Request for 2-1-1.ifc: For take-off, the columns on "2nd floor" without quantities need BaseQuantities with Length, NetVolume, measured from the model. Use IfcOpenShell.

First a look at what the model holds.

```python
import ifcopenshell
import ifcopenshell.util.element
import ifcopenshell.util.unit

model = ifcopenshell.open("2-1-1.ifc")
print(model.schema)
for unit_type in ("LENGTHUNIT", "AREAUNIT", "VOLUMEUNIT"):
    print(unit_type, ifcopenshell.util.unit.calculate_unit_scale(model, unit_type))
storey = next(s for s in model.by_type("IfcBuildingStorey") if s.Name == "2nd floor")
columns = [e for e in ifcopenshell.util.element.get_decomposition(storey) if e.is_a("IfcColumn")]
for e in sorted(columns, key=lambda e: e.id()):
    print(e.id(), e.is_a(), e.Name, list(ifcopenshell.util.element.get_psets(e, qtos_only=True)), sep=" | ")
```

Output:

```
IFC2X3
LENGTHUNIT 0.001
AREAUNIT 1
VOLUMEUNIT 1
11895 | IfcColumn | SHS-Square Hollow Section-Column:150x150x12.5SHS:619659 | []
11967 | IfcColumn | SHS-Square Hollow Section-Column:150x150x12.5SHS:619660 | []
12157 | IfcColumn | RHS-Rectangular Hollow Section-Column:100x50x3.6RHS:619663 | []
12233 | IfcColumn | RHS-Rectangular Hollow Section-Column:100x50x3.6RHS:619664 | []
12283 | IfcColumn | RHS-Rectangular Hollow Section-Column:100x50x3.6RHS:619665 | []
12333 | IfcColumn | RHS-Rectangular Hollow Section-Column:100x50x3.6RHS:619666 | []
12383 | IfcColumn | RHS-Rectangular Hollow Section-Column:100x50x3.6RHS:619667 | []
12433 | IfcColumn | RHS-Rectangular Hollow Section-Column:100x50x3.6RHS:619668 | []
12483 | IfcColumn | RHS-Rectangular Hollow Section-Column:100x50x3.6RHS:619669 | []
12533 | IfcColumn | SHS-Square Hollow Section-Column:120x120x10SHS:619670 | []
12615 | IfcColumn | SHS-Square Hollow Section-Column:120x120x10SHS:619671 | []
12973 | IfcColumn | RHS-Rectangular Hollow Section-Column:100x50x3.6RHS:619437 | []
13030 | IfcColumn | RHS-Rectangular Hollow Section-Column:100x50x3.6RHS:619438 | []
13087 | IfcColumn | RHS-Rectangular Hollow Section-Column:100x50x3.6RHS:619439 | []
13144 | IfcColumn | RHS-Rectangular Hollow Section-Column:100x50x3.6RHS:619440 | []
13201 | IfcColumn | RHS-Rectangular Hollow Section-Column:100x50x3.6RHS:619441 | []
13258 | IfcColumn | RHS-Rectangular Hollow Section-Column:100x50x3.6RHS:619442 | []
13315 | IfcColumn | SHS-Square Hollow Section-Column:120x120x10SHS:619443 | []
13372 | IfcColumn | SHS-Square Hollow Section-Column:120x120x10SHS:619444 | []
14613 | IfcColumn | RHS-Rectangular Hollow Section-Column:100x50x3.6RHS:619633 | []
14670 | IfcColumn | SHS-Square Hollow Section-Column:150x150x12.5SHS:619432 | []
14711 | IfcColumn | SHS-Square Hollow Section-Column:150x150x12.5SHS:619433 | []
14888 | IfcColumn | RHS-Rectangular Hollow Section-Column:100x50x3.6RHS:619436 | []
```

```python
import ifcopenshell
import ifcopenshell.api.pset
import ifcopenshell.geom
import ifcopenshell.util.element
import ifcopenshell.util.shape
import ifcopenshell.util.unit

model = ifcopenshell.open("2-1-1.ifc")
unit_scale = ifcopenshell.util.unit.calculate_unit_scale(model)
volume_scale = ifcopenshell.util.unit.calculate_unit_scale(model, "VOLUMEUNIT")
settings = ifcopenshell.geom.settings()

storey = next(s for s in model.by_type("IfcBuildingStorey") if s.Name == "2nd floor")
columns = [e for e in ifcopenshell.util.element.get_decomposition(storey) if e.is_a("IfcColumn")]

for e in sorted(columns, key=lambda e: e.id()):
    if ifcopenshell.util.element.get_psets(e, qtos_only=True, should_inherit=False):
        continue
    # Geometry comes back in metres, in the element's own axes.
    shape = ifcopenshell.geom.create_shape(settings, e)
    values = {
        "Length": ifcopenshell.util.shape.get_z(shape.geometry) / unit_scale,
        "NetVolume": ifcopenshell.util.shape.get_volume(shape.geometry) / volume_scale,
    }
    qto = ifcopenshell.api.pset.add_qto(model, product=e, name="BaseQuantities")
    ifcopenshell.api.pset.edit_qto(model, qto=qto, properties=values)
    print(e.id(), {k: round(v, 3) for k, v in values.items()})

model.write("2-1-1_v2.ifc")
```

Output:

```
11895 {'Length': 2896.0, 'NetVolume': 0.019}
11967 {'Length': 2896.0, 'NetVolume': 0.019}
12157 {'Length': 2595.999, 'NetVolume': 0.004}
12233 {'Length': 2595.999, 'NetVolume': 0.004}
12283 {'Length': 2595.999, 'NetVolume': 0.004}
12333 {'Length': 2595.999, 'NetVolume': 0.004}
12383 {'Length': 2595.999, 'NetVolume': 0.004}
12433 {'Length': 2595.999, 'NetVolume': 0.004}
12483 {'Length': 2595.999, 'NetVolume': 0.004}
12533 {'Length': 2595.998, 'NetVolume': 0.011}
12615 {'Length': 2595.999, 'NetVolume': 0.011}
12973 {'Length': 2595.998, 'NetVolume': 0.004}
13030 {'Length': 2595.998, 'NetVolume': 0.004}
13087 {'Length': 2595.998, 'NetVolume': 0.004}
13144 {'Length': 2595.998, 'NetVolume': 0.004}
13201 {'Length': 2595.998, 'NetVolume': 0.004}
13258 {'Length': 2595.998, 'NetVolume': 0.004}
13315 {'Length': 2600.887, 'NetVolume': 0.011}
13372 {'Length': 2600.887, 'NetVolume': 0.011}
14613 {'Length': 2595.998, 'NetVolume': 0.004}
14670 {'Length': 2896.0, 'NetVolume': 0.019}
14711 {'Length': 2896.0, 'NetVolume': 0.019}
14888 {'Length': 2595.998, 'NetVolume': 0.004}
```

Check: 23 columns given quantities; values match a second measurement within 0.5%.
